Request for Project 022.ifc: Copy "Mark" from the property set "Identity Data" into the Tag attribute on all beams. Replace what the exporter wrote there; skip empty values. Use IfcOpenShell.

First a look at what the model holds.

```python
import ifcopenshell
import ifcopenshell.util.element

model = ifcopenshell.open("Project 022.ifc")
print(model.schema)
beams = model.by_type("IfcBeam")
print(len(beams), "beams")
for e in beams[:8]:
    source = ifcopenshell.util.element.get_pset(e, "Identity Data", "Mark")
    target = e.Tag
    print(e.id(), repr(source), repr(target), sep=" | ")
```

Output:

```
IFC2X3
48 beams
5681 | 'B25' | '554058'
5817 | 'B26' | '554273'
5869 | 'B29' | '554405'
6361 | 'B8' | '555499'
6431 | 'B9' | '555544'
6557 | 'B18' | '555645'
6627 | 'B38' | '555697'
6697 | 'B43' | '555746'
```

```python
import ifcopenshell
import ifcopenshell.util.element

model = ifcopenshell.open("Project 022.ifc")

count = 0
for e in model.by_type("IfcBeam"):
    value = ifcopenshell.util.element.get_pset(e, "Identity Data", "Mark")
    current = e.Tag
    if not value or not value.strip() or current == value:
        continue
    e.Tag = value
    count += 1

print(count, "beams updated")

model.write("Project 022_v2.ifc")
```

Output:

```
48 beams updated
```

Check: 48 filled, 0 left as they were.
